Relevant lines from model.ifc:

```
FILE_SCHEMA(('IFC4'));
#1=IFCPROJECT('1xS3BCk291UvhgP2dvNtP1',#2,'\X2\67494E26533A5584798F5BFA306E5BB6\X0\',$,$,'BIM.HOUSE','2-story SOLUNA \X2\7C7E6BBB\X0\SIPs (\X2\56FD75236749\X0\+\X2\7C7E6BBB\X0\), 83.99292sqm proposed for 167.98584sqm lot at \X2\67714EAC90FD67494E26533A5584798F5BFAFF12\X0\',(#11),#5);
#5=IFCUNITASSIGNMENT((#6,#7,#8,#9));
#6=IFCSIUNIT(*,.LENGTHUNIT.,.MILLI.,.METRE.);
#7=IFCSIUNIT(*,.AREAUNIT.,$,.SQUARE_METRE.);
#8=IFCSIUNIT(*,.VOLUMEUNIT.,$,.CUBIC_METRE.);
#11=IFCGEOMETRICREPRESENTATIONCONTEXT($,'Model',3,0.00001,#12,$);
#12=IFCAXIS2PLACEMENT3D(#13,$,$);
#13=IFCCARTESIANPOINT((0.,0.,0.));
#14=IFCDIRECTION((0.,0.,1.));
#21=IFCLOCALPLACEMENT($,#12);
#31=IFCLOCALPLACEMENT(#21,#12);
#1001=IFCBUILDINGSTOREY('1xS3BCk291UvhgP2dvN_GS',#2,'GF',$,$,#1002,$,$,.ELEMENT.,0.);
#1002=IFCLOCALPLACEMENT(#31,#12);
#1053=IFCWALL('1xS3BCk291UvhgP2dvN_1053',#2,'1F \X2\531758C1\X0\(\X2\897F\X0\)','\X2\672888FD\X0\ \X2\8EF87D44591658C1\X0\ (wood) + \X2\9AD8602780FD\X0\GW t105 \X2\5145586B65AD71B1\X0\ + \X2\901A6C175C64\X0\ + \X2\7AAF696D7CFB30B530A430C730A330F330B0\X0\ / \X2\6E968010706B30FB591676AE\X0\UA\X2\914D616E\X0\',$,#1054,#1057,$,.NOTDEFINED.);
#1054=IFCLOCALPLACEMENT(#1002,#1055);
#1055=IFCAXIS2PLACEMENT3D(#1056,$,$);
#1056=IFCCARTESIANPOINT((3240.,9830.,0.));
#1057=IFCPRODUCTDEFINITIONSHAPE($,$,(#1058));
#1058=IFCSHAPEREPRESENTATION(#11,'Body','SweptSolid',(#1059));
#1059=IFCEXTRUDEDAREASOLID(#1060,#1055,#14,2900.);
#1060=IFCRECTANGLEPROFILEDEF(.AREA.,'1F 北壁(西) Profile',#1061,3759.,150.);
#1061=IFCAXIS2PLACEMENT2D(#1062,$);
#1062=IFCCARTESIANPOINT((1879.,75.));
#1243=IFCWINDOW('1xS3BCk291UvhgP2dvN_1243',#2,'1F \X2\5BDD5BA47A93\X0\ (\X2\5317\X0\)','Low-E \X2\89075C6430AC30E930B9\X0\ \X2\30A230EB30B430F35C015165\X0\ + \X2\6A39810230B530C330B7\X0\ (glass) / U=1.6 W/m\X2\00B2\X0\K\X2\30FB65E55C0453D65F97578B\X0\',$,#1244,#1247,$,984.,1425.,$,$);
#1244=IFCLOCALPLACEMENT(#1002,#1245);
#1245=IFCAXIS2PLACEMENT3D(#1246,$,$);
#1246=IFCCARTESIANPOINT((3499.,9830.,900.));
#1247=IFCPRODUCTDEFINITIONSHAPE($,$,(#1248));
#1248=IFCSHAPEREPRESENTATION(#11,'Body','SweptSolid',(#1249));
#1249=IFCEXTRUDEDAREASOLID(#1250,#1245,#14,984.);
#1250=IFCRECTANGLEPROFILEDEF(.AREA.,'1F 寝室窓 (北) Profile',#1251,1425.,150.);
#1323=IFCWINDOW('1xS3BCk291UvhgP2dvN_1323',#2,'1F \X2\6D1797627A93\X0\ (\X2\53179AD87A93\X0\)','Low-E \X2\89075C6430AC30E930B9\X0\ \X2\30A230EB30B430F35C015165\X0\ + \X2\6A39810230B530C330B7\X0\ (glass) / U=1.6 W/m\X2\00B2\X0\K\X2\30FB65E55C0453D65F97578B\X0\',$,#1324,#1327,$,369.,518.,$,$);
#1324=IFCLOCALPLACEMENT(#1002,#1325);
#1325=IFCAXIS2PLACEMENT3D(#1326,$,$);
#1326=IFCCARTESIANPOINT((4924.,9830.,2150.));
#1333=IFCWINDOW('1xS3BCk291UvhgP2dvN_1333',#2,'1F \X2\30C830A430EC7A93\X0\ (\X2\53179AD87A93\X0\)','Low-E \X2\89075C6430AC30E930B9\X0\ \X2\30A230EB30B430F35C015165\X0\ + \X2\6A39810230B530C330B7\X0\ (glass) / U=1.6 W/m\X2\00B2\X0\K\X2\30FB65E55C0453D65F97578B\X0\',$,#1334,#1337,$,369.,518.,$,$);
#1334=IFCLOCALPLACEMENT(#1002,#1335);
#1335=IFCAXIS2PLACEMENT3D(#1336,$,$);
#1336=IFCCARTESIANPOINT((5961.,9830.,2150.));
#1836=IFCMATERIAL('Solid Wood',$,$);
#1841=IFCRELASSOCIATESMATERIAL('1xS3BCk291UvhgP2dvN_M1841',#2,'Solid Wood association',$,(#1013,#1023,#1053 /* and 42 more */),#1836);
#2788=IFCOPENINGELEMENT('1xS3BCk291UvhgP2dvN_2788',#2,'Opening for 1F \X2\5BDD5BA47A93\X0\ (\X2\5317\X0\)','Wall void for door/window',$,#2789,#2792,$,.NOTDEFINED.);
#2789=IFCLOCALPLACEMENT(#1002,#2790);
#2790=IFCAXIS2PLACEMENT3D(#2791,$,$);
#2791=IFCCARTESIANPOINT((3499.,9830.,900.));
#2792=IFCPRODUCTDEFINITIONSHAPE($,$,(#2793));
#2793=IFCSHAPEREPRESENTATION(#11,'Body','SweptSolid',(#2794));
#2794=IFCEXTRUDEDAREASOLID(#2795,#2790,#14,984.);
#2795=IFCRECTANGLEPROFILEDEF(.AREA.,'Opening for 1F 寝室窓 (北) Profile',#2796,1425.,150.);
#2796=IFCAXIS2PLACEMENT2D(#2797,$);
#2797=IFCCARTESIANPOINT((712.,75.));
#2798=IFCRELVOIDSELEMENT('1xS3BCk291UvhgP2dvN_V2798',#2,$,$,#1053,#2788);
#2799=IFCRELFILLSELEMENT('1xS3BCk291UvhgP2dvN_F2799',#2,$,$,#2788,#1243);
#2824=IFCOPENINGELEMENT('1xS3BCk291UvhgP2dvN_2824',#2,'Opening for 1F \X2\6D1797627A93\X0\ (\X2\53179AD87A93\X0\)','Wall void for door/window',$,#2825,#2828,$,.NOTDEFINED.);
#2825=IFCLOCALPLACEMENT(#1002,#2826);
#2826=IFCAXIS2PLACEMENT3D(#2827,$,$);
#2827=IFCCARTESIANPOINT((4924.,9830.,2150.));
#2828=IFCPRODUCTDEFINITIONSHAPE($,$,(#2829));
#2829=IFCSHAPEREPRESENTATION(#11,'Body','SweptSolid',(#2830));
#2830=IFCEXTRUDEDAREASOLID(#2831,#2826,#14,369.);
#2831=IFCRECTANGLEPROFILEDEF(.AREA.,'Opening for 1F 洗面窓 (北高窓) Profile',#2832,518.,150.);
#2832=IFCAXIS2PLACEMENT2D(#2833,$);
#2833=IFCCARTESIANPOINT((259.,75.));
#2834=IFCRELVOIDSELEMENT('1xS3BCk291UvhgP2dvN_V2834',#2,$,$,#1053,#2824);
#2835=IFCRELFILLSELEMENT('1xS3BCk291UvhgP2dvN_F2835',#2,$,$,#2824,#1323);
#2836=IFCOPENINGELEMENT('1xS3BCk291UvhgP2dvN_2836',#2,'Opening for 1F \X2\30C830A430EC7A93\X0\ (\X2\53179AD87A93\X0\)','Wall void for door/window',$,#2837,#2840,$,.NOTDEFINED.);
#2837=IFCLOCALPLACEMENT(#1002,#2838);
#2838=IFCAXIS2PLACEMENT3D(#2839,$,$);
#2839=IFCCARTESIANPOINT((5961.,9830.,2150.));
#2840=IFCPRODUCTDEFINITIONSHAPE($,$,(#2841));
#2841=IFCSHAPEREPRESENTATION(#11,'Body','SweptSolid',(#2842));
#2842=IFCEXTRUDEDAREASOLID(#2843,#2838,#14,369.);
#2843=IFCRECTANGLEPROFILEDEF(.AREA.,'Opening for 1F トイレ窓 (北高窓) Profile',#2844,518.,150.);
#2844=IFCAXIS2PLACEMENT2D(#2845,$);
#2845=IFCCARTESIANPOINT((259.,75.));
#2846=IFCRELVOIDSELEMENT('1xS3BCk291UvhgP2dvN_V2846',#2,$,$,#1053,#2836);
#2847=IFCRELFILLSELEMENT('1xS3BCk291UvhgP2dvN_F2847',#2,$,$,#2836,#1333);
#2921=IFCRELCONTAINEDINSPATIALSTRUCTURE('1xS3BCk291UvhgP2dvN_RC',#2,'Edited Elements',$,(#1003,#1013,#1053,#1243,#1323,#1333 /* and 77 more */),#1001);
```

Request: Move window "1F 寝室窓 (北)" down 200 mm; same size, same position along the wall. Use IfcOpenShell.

```python
import numpy as np
import ifcopenshell
import ifcopenshell.api.geometry
import ifcopenshell.util.placement
import ifcopenshell.util.unit

model = ifcopenshell.open("model.ifc")
unit_scale = ifcopenshell.util.unit.calculate_unit_scale(model)

window = model.by_id(1243)
opening = window.FillsVoids[0].RelatingOpeningElement
dz = -0.2 / unit_scale

shift = np.array([0.0, 0.0, dz])
# The window is not placed relative to its opening, so move both.
for product in (opening, window):
    matrix = ifcopenshell.util.placement.get_local_placement(product.ObjectPlacement)
    matrix[:3, 3] += shift
    ifcopenshell.api.geometry.edit_object_placement(model, product=product, matrix=matrix, is_si=False)

print(f"moved by {dz * unit_scale:+.3f} m")

model.write("model_v2.ifc")
```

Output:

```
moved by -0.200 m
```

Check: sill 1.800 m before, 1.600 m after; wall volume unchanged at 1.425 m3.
